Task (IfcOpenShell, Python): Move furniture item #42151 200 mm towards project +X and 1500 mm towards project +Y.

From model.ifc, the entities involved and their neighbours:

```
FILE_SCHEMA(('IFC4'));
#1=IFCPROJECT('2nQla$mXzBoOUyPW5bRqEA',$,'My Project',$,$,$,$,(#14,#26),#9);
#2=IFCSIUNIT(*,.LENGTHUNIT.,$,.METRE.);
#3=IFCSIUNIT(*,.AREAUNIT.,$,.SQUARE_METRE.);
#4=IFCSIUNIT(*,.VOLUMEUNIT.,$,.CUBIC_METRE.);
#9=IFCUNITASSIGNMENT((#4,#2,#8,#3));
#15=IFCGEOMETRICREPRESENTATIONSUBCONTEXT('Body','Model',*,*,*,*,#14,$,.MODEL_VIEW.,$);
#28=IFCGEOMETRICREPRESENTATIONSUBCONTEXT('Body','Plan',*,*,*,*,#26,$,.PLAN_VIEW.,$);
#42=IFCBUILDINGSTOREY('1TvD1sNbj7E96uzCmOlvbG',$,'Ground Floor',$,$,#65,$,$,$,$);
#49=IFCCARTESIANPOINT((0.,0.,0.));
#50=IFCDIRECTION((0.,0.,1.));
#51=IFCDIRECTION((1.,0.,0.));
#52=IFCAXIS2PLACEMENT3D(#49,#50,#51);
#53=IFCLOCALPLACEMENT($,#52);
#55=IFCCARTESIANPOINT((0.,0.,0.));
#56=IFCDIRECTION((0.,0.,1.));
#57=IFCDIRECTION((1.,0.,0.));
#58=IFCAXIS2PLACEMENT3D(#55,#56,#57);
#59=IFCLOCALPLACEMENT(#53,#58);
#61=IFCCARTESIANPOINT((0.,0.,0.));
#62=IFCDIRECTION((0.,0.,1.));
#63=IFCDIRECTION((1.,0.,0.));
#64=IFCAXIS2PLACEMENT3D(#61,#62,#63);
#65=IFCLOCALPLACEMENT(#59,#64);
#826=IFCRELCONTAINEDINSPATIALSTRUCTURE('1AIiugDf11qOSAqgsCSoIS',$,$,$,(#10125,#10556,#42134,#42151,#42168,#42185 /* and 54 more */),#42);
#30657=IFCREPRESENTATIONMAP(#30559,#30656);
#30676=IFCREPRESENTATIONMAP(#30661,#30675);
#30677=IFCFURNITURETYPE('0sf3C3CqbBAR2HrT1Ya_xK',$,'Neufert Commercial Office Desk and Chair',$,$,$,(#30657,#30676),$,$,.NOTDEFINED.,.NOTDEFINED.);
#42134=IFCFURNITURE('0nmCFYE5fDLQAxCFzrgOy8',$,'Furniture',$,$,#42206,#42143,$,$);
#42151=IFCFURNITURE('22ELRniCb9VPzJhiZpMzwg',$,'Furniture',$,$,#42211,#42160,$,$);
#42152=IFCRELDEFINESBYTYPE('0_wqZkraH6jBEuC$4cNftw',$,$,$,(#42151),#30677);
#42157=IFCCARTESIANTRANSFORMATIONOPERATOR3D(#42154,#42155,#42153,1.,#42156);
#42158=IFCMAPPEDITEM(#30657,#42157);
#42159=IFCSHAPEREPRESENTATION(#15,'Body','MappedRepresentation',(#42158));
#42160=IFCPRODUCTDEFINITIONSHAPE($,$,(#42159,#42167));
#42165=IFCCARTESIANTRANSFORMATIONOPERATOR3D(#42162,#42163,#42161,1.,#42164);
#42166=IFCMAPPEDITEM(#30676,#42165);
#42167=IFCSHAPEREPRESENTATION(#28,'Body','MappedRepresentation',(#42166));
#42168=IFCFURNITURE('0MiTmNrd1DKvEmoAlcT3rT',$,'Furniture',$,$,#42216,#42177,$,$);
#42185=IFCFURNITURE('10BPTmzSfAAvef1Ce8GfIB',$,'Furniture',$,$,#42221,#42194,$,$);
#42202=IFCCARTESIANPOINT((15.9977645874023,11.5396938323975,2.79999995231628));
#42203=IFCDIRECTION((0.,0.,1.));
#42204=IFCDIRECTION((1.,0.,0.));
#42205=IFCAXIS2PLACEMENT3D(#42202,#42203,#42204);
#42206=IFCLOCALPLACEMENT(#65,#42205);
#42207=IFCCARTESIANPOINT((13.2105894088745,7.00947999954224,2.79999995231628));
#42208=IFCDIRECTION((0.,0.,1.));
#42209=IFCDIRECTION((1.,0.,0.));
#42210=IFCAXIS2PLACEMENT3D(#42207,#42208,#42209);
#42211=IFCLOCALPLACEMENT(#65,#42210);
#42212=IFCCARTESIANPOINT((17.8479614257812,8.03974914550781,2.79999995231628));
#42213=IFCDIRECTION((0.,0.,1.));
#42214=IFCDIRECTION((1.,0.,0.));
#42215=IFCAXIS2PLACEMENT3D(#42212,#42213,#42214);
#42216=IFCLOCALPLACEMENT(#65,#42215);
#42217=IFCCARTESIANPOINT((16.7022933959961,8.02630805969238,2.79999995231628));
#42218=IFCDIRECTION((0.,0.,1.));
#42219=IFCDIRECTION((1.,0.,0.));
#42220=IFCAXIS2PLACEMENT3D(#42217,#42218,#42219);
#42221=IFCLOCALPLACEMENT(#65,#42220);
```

```python
import ifcopenshell
import ifcopenshell.api.geometry
import ifcopenshell.util.placement
import ifcopenshell.util.unit

model = ifcopenshell.open("model.ifc")
unit_scale = ifcopenshell.util.unit.calculate_unit_scale(model)

item = model.by_guid("22ELRniCb9VPzJhiZpMzwg")
matrix = ifcopenshell.util.placement.get_local_placement(item.ObjectPlacement)
matrix[0, 3] += 0.2 / unit_scale
matrix[1, 3] += 1.5 / unit_scale
ifcopenshell.api.geometry.edit_object_placement(model, product=item, matrix=matrix, is_si=False)

print(ifcopenshell.util.placement.get_local_placement(item.ObjectPlacement).round(3) + 0.0)

model.write("model_v2.ifc")
```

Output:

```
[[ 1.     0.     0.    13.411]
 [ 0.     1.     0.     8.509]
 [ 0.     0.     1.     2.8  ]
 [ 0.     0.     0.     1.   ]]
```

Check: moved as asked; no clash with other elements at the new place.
